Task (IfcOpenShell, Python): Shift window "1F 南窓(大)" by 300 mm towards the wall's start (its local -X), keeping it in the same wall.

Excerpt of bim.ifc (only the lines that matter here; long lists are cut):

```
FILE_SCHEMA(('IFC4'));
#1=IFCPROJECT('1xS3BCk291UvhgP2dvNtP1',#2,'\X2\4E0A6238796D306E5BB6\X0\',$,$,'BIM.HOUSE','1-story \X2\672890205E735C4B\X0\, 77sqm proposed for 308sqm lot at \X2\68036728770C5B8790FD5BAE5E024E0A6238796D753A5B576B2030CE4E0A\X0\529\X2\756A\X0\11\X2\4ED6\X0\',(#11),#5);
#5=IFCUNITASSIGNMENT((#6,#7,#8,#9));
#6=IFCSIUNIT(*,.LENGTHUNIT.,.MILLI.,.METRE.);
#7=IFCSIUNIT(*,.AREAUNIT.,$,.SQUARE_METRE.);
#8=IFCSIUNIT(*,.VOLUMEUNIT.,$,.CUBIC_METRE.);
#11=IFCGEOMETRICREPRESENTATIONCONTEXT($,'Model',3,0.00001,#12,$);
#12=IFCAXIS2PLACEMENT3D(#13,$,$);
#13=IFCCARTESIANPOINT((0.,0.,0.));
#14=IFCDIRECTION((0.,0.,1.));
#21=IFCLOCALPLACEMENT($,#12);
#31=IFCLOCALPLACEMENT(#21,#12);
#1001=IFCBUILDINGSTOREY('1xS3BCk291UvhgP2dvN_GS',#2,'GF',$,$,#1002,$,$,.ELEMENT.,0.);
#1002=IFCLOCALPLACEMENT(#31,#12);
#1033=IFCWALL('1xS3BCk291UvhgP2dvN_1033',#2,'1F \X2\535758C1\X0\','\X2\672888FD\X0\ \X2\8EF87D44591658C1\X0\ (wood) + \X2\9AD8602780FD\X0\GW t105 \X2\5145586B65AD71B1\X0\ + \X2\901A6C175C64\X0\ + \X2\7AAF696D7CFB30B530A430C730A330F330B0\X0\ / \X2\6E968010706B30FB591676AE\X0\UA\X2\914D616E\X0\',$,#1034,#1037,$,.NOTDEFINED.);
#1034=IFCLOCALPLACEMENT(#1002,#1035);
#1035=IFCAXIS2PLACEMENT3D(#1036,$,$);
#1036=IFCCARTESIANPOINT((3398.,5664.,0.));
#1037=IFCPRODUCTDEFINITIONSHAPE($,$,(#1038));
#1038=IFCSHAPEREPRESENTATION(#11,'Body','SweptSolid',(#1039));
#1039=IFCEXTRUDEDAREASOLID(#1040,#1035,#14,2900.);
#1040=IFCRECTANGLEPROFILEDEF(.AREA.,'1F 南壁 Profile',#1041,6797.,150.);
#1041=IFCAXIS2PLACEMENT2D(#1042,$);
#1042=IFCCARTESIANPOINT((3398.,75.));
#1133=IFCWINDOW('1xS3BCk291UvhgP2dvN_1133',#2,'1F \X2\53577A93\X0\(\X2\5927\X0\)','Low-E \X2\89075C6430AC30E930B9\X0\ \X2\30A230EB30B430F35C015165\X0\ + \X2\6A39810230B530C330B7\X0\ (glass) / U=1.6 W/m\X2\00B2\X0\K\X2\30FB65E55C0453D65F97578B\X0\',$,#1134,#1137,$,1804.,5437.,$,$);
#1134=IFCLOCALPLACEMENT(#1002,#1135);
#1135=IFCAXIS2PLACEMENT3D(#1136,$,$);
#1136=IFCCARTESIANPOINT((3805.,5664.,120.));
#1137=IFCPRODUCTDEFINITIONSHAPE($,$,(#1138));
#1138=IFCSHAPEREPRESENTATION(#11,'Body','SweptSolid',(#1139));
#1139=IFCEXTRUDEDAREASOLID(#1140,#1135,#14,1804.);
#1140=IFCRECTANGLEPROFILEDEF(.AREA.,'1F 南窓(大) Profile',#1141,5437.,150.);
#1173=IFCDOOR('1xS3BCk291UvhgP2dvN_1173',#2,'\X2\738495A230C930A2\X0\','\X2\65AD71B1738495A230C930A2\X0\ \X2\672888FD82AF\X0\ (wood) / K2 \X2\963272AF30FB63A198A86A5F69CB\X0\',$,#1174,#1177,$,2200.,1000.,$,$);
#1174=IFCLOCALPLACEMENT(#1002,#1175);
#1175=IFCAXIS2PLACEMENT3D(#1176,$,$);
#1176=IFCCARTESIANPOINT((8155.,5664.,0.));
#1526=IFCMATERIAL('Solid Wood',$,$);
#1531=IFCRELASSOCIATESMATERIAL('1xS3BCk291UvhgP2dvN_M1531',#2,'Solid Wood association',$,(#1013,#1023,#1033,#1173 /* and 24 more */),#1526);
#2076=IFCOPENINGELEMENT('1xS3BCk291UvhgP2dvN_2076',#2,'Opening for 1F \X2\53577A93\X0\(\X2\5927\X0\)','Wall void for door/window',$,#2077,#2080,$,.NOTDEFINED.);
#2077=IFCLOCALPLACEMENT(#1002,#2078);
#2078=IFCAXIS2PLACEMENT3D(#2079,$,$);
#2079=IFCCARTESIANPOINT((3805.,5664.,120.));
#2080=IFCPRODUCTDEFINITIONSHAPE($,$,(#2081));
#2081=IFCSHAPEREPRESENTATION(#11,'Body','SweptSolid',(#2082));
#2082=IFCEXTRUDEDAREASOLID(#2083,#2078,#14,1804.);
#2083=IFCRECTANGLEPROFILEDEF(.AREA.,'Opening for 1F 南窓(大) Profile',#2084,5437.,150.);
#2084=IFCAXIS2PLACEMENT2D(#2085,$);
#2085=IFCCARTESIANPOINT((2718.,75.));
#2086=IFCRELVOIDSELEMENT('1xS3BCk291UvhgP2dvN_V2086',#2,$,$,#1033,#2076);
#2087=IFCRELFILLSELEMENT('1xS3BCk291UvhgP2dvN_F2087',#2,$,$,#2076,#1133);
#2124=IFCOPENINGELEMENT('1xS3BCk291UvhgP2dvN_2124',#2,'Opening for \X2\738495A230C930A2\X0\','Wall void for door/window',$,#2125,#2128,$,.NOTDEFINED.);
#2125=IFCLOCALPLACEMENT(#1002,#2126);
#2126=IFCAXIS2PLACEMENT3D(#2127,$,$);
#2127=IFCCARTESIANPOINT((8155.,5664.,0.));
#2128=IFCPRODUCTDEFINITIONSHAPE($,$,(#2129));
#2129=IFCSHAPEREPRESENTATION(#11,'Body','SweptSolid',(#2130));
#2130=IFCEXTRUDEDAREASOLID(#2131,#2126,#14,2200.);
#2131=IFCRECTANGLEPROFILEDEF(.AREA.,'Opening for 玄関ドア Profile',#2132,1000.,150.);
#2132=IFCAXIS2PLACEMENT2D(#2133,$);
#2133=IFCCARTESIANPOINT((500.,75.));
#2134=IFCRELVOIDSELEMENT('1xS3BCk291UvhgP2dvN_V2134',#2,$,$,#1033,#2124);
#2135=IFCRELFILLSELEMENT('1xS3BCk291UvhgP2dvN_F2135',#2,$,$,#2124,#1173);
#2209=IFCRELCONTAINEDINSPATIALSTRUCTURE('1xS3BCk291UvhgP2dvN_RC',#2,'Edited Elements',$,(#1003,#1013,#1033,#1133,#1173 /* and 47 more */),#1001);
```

```python
import ifcopenshell
import ifcopenshell.api.geometry
import ifcopenshell.util.placement
import ifcopenshell.util.unit

model = ifcopenshell.open("bim.ifc")
unit_scale = ifcopenshell.util.unit.calculate_unit_scale(model)

window = model.by_guid("1xS3BCk291UvhgP2dvN_1133")
opening = window.FillsVoids[0].RelatingOpeningElement
wall = opening.VoidsElements[0].RelatingBuildingElement

wall_matrix = ifcopenshell.util.placement.get_local_placement(wall.ObjectPlacement)
shift = wall_matrix[:3, 0] * -0.3 / unit_scale
before = ifcopenshell.util.placement.get_local_placement(window.ObjectPlacement)[:3, 3].copy()

# The window is not placed relative to its opening, so move both.
for product in (opening, window):
    matrix = ifcopenshell.util.placement.get_local_placement(product.ObjectPlacement)
    matrix[:3, 3] += shift
    ifcopenshell.api.geometry.edit_object_placement(model, product=product, matrix=matrix, is_si=False)

after = ifcopenshell.util.placement.get_local_placement(window.ObjectPlacement)[:3, 3]
print("window moved by", (after - before).round(3) + 0.0)

model.write("bim_updated.ifc")
```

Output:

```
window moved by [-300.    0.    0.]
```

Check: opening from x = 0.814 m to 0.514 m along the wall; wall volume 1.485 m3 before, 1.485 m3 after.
